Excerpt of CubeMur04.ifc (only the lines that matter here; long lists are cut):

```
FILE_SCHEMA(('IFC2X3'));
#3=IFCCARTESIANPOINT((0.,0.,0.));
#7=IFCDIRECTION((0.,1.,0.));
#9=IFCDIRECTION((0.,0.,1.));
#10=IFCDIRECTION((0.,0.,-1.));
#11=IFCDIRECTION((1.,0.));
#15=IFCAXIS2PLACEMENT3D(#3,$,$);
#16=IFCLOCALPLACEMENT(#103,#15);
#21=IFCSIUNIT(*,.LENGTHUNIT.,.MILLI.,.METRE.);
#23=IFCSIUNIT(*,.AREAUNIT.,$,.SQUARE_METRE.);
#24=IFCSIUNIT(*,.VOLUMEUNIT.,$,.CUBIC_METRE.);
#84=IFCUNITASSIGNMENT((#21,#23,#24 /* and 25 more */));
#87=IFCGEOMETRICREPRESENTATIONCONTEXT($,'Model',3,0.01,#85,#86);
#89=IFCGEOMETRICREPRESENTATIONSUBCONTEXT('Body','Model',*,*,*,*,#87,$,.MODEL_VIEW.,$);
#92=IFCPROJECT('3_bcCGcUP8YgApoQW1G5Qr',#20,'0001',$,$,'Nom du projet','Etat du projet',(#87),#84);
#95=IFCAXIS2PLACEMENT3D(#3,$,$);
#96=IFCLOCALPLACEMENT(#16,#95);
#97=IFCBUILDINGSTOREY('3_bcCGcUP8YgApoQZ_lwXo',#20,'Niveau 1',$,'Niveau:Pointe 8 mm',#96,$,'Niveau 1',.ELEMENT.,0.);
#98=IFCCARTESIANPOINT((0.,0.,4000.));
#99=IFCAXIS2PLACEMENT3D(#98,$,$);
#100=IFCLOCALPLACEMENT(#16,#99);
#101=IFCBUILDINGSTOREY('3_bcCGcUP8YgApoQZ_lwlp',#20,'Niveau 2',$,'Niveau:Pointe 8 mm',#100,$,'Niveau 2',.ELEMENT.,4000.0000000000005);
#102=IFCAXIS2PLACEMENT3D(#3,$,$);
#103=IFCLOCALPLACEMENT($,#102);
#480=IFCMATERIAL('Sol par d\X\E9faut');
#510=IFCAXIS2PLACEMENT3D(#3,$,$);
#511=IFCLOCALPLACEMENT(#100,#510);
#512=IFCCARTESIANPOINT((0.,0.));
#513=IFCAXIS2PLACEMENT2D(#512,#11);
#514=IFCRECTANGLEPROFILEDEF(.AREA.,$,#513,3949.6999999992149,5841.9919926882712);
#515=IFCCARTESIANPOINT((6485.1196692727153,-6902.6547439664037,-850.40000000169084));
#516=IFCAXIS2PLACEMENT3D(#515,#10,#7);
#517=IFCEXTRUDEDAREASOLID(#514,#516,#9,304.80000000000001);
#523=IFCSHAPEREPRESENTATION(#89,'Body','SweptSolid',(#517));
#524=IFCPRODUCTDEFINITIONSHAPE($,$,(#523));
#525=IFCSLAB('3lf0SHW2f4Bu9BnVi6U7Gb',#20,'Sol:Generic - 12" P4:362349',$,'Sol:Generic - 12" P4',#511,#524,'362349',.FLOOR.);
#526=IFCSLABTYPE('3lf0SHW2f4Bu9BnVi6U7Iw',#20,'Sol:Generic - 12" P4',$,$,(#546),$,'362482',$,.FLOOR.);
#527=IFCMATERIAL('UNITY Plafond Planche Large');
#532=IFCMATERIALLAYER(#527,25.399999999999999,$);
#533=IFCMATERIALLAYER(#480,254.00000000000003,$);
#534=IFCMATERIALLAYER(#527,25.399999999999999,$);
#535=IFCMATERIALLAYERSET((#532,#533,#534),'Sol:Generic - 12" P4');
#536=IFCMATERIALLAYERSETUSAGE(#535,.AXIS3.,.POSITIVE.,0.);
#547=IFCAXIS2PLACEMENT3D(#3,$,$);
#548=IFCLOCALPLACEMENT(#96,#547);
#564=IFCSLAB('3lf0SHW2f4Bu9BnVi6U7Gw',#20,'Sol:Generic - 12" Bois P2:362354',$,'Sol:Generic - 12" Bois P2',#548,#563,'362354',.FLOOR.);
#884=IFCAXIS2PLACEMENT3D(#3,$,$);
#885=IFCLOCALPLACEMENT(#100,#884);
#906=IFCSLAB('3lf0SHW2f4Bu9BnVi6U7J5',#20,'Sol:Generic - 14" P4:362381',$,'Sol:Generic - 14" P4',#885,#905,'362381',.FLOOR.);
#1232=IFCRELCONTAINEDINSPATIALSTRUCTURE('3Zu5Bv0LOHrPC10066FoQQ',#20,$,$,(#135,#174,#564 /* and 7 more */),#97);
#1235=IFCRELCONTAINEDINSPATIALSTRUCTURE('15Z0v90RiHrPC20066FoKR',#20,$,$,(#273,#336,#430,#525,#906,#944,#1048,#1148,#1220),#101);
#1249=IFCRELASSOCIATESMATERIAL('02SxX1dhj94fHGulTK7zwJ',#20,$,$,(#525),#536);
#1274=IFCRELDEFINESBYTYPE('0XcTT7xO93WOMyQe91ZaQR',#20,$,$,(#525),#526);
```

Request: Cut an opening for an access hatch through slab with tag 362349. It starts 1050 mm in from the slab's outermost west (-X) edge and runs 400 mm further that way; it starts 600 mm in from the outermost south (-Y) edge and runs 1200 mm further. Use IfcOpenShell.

```python
import numpy as np
import ifcopenshell
import ifcopenshell.api.feature
import ifcopenshell.api.geometry
import ifcopenshell.api.root
import ifcopenshell.geom
import ifcopenshell.util.placement
import ifcopenshell.util.representation
import ifcopenshell.util.shape
import ifcopenshell.util.unit

model = ifcopenshell.open("CubeMur04.ifc")
unit_scale = ifcopenshell.util.unit.calculate_unit_scale(model)
settings = ifcopenshell.geom.settings()


def volume(element):
    """Net volume in cubic metres, openings subtracted."""
    shape = ifcopenshell.geom.create_shape(settings, element)
    return ifcopenshell.util.shape.get_volume(shape.geometry)


slab = model.by_guid("3lf0SHW2f4Bu9BnVi6U7Gb")
before = volume(slab)

# Extent in the slab's own axes, in metres. The edges named are its -X and -Y sides.
slab_shape = ifcopenshell.geom.create_shape(settings, slab)
vertices = ifcopenshell.util.shape.get_vertices(slab_shape.geometry)
x_min, y_min, bottom = vertices.min(axis=0)
top = vertices[:, 2].max()

opening = ifcopenshell.api.root.create_entity(model, ifc_class="IfcOpeningElement", name="Access hatch opening")
context = ifcopenshell.util.representation.get_context(model, "Model", "Body", "MODEL_VIEW")
width, depth = 0.4, 1.2
outline = [(0.0, 0.0), (width, 0.0), (width, depth), (0.0, depth), (0.0, 0.0)]
# Overshoot both faces by 50 mm so the cut is clean.
shape = ifcopenshell.api.geometry.add_slab_representation(
    model, context=context, depth=top - bottom + 0.1, polyline=outline
)
ifcopenshell.api.geometry.assign_representation(model, product=opening, representation=shape)

matrix = ifcopenshell.util.placement.get_local_placement(slab.ObjectPlacement)
matrix[:, 3] = matrix @ np.append(np.array([x_min + 1.05, y_min + 0.6, bottom - 0.05]) / unit_scale, 1.0)
ifcopenshell.api.geometry.edit_object_placement(model, product=opening, matrix=matrix, is_si=False)
ifcopenshell.api.feature.add_feature(model, feature=opening, element=slab)

after = volume(slab)

print(f"slab volume {before:.3f} -> {after:.3f} m3")

model.write("CubeMur04_edited.ifc")
```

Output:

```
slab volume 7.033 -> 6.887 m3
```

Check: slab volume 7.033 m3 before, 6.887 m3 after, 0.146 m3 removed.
